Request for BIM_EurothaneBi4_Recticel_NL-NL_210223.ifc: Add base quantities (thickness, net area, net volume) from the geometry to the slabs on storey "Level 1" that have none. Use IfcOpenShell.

First a look at what the model holds.

```python
import ifcopenshell
import ifcopenshell.util.element
import ifcopenshell.util.unit

model = ifcopenshell.open("BIM_EurothaneBi4_Recticel_NL-NL_210223.ifc")
print(model.schema)
for unit_type in ("LENGTHUNIT", "AREAUNIT", "VOLUMEUNIT"):
    print(unit_type, ifcopenshell.util.unit.calculate_unit_scale(model, unit_type))
storey = next(s for s in model.by_type("IfcBuildingStorey") if s.Name == "Level 1")
slabs = [e for e in ifcopenshell.util.element.get_decomposition(storey) if e.is_a("IfcSlab")]
for e in sorted(slabs, key=lambda e: e.id()):
    print(e.id(), e.is_a(), e.Name, list(ifcopenshell.util.element.get_psets(e, qtos_only=True)), sep=" | ")
```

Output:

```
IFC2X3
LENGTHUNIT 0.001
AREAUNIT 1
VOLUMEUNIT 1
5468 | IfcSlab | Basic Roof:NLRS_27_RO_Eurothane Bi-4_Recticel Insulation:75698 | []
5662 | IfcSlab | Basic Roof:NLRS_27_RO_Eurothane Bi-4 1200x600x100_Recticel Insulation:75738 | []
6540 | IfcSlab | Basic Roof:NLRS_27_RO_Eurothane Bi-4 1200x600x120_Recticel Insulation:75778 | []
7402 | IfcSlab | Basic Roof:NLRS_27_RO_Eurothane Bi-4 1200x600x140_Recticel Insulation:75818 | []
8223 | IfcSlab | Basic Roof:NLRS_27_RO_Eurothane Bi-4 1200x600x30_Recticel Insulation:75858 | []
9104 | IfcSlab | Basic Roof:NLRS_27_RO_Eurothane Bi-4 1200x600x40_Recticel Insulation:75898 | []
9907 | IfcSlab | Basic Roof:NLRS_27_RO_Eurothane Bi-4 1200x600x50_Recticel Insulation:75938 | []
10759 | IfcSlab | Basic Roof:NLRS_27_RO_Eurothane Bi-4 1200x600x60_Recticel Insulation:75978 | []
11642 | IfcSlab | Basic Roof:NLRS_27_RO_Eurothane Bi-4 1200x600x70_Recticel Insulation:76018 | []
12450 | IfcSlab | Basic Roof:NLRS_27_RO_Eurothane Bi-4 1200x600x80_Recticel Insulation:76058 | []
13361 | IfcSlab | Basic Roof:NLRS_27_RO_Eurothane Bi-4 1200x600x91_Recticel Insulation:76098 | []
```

```python
import ifcopenshell
import ifcopenshell.api.pset
import ifcopenshell.geom
import ifcopenshell.util.element
import ifcopenshell.util.shape
import ifcopenshell.util.unit

model = ifcopenshell.open("BIM_EurothaneBi4_Recticel_NL-NL_210223.ifc")
unit_scale = ifcopenshell.util.unit.calculate_unit_scale(model)
area_scale = ifcopenshell.util.unit.calculate_unit_scale(model, "AREAUNIT")
volume_scale = ifcopenshell.util.unit.calculate_unit_scale(model, "VOLUMEUNIT")
settings = ifcopenshell.geom.settings()

storey = next(s for s in model.by_type("IfcBuildingStorey") if s.Name == "Level 1")
slabs = [e for e in ifcopenshell.util.element.get_decomposition(storey) if e.is_a("IfcSlab")]

for e in sorted(slabs, key=lambda e: e.id()):
    if ifcopenshell.util.element.get_psets(e, qtos_only=True, should_inherit=False):
        continue
    # Geometry comes back in metres, in the element's own axes.
    shape = ifcopenshell.geom.create_shape(settings, e)
    values = {
        "Width": ifcopenshell.util.shape.get_z(shape.geometry) / unit_scale,
        "NetArea": ifcopenshell.util.shape.get_footprint_area(shape.geometry) / area_scale,
        "NetVolume": ifcopenshell.util.shape.get_volume(shape.geometry) / volume_scale,
    }
    qto = ifcopenshell.api.pset.add_qto(model, product=e, name="BaseQuantities")
    ifcopenshell.api.pset.edit_qto(model, qto=qto, properties=values)
    print(e.id(), {k: round(v, 3) for k, v in values.items()})

model.write("BIM_EurothaneBi4_Recticel_NL-NL_210223-out.ifc")
```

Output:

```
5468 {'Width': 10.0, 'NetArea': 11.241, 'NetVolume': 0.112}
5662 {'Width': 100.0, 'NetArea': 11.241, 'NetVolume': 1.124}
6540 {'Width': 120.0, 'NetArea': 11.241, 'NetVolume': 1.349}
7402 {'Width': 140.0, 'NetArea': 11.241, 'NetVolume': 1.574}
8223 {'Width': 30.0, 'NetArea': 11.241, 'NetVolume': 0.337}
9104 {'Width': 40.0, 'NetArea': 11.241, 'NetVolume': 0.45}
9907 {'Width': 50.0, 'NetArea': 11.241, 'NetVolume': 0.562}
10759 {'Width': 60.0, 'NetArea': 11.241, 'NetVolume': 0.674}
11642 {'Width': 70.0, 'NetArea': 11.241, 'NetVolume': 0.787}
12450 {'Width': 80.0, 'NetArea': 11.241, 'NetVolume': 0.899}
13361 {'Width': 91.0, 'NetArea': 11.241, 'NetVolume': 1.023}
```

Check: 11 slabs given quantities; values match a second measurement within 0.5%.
